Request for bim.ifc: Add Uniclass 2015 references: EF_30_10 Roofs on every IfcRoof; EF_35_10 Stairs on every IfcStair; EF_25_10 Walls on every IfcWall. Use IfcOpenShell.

First a look at what the model holds.

```python
import ifcopenshell

model = ifcopenshell.open("bim.ifc")
print(model.schema)
print("classifications:", [c.Name for c in model.by_type("IfcClassification")])
for ifc_class in ("IfcDoor", "IfcRoof", "IfcStair", "IfcWall", "IfcWindow"):
    print(ifc_class, len(model.by_type(ifc_class)))
```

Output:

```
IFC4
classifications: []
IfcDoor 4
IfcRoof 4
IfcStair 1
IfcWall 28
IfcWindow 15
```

```python
import ifcopenshell
import ifcopenshell.api.classification

model = ifcopenshell.open("bim.ifc")

system = ifcopenshell.api.classification.add_classification(model, classification="Uniclass 2015")

codes = {
    "IfcRoof": ("EF_30_10", "Roofs"),
    "IfcStair": ("EF_35_10", "Stairs"),
    "IfcWall": ("EF_25_10", "Walls"),
}
for ifc_class, (code, name) in codes.items():
    products = model.by_type(ifc_class)
    ifcopenshell.api.classification.add_reference(
        model, products=products, classification=system, identification=code, name=name
    )
    print(code, len(products))

model.write("bim-out.ifc")
```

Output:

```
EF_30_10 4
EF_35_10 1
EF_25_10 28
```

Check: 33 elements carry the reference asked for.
